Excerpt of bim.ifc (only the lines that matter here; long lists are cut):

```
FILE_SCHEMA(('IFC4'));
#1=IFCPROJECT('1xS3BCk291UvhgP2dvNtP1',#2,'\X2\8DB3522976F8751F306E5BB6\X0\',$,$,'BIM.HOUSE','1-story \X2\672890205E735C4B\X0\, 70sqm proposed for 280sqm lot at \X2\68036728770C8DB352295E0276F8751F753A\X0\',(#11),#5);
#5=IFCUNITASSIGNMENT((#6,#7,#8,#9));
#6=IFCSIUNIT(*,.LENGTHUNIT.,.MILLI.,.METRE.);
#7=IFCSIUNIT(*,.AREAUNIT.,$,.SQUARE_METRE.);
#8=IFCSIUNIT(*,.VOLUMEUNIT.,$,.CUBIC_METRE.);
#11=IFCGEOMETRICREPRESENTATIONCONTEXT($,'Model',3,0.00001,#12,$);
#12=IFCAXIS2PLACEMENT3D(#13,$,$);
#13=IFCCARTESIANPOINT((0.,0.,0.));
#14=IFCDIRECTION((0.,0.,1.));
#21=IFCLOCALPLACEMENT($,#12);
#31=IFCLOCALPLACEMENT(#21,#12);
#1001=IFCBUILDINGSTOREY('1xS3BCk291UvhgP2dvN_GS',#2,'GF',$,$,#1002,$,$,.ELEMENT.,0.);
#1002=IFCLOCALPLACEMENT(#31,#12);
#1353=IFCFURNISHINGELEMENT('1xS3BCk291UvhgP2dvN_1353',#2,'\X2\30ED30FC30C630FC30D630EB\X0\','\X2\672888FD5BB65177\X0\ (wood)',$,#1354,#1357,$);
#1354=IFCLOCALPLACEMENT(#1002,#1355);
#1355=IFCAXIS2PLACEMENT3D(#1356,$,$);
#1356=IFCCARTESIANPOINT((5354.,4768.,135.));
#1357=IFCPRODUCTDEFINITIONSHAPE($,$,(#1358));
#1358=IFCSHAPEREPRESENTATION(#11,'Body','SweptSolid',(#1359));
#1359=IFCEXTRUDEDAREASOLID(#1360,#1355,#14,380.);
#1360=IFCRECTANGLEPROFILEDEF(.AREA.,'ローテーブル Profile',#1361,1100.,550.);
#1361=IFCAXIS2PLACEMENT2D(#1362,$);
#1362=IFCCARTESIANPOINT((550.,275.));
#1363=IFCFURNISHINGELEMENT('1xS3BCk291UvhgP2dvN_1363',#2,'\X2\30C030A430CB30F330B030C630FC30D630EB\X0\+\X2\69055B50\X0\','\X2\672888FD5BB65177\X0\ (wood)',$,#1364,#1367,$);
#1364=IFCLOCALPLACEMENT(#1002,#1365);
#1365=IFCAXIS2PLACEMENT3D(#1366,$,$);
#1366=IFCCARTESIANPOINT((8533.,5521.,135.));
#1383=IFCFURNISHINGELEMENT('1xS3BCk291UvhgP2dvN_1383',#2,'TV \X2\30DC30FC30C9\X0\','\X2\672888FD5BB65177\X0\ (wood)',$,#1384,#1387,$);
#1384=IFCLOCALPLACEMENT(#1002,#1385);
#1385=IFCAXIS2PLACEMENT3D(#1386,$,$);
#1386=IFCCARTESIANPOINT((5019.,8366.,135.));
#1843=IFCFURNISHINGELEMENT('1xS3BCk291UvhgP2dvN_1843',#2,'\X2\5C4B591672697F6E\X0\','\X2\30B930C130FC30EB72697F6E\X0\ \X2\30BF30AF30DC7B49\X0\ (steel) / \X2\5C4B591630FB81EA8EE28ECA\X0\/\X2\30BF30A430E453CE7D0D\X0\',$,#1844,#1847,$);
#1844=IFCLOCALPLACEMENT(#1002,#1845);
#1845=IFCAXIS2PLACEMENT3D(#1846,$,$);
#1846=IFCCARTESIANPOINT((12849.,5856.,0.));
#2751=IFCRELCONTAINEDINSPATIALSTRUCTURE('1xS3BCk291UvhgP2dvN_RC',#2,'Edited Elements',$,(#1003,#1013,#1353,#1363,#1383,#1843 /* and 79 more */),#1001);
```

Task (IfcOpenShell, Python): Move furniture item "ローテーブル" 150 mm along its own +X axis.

```python
import ifcopenshell
import ifcopenshell.api.geometry
import ifcopenshell.util.placement
import ifcopenshell.util.unit

model = ifcopenshell.open("bim.ifc")
unit_scale = ifcopenshell.util.unit.calculate_unit_scale(model)

item = model.by_guid("1xS3BCk291UvhgP2dvN_1353")
matrix = ifcopenshell.util.placement.get_local_placement(item.ObjectPlacement)
matrix[:3, 3] += matrix[:3, 0] * 0.15 / unit_scale
ifcopenshell.api.geometry.edit_object_placement(model, product=item, matrix=matrix, is_si=False)

print(ifcopenshell.util.placement.get_local_placement(item.ObjectPlacement).round(3) + 0.0)

model.write("bim_updated.ifc")
```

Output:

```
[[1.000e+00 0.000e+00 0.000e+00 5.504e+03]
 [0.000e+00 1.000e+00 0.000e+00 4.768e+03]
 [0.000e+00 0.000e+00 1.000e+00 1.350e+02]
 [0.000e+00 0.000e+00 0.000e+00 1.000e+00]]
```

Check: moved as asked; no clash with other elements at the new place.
